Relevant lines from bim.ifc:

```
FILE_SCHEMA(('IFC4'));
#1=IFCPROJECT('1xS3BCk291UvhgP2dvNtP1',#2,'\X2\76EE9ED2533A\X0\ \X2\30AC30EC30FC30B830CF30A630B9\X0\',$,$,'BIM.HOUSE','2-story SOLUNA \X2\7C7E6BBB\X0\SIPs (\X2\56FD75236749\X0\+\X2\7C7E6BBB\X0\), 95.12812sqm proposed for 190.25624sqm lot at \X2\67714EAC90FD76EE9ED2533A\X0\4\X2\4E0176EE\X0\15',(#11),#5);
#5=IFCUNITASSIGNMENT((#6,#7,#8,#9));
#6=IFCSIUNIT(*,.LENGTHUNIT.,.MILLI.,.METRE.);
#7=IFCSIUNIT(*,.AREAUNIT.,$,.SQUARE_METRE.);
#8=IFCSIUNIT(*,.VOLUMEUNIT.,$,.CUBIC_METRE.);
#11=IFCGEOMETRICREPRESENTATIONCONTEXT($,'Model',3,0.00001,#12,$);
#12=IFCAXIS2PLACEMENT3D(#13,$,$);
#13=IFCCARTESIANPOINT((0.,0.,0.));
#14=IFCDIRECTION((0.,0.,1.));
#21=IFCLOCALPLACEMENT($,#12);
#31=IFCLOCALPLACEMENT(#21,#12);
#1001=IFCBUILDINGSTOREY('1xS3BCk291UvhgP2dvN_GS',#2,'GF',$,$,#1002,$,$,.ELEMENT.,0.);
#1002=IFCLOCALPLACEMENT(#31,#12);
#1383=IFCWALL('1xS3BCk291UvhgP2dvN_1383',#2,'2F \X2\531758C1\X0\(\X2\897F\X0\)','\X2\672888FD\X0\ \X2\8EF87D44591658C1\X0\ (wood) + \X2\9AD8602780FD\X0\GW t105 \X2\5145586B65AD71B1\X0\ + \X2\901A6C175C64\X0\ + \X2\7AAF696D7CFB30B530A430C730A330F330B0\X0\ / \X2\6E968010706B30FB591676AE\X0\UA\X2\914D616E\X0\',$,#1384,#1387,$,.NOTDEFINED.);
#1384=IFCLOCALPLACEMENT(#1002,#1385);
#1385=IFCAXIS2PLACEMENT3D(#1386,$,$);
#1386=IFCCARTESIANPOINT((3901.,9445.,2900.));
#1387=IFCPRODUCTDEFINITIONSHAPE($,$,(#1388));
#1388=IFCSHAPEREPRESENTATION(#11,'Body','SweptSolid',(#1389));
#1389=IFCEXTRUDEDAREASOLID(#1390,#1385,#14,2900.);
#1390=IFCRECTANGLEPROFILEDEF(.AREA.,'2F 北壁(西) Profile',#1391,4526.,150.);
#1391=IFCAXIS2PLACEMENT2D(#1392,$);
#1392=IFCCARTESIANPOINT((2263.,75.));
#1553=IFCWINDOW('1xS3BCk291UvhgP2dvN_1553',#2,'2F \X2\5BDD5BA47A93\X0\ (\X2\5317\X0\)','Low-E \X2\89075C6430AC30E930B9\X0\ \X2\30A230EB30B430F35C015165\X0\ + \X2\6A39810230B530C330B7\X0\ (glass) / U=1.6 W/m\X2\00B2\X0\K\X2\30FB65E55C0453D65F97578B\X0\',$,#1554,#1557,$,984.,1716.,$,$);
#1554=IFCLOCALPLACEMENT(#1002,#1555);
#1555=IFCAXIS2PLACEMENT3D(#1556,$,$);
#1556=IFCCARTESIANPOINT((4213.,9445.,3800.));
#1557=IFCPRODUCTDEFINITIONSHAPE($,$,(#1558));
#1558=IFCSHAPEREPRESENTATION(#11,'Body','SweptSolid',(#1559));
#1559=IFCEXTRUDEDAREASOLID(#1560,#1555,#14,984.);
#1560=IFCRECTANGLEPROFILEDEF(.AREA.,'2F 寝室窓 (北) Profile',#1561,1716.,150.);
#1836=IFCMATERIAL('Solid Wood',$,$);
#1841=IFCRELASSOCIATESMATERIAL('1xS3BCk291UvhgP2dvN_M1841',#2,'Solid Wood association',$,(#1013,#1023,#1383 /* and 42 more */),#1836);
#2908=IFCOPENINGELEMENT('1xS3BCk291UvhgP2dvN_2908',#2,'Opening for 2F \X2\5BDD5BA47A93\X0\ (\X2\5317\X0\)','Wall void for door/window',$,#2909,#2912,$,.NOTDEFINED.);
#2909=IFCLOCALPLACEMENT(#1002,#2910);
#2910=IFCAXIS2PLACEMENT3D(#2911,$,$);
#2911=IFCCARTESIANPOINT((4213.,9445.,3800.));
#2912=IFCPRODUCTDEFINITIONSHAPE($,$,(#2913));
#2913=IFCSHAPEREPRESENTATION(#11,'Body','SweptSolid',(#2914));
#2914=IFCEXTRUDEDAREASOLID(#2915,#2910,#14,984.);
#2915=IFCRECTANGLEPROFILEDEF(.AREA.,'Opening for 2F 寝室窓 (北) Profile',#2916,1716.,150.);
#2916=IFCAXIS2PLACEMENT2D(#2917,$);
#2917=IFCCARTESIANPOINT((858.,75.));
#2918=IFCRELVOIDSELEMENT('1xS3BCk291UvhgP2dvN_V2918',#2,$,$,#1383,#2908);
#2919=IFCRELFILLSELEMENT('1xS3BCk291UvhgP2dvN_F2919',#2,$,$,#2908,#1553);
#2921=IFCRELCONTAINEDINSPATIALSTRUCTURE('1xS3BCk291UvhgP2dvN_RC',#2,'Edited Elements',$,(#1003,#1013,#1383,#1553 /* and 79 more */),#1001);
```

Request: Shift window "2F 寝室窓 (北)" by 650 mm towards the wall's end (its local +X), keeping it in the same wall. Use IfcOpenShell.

```python
import ifcopenshell
import ifcopenshell.api.geometry
import ifcopenshell.util.placement
import ifcopenshell.util.unit

model = ifcopenshell.open("bim.ifc")
unit_scale = ifcopenshell.util.unit.calculate_unit_scale(model)

window = model.by_guid("1xS3BCk291UvhgP2dvN_1553")
opening = window.FillsVoids[0].RelatingOpeningElement
wall = opening.VoidsElements[0].RelatingBuildingElement

wall_matrix = ifcopenshell.util.placement.get_local_placement(wall.ObjectPlacement)
shift = wall_matrix[:3, 0] * 0.65 / unit_scale
before = ifcopenshell.util.placement.get_local_placement(window.ObjectPlacement)[:3, 3].copy()

# The window is not placed relative to its opening, so move both.
for product in (opening, window):
    matrix = ifcopenshell.util.placement.get_local_placement(product.ObjectPlacement)
    matrix[:3, 3] += shift
    ifcopenshell.api.geometry.edit_object_placement(model, product=product, matrix=matrix, is_si=False)

after = ifcopenshell.util.placement.get_local_placement(window.ObjectPlacement)[:3, 3]
print("window moved by", (after - before).round(3) + 0.0)

model.write("bim_updated.ifc")
```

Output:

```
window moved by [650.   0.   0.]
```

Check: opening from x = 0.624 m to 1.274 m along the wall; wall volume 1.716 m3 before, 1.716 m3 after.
